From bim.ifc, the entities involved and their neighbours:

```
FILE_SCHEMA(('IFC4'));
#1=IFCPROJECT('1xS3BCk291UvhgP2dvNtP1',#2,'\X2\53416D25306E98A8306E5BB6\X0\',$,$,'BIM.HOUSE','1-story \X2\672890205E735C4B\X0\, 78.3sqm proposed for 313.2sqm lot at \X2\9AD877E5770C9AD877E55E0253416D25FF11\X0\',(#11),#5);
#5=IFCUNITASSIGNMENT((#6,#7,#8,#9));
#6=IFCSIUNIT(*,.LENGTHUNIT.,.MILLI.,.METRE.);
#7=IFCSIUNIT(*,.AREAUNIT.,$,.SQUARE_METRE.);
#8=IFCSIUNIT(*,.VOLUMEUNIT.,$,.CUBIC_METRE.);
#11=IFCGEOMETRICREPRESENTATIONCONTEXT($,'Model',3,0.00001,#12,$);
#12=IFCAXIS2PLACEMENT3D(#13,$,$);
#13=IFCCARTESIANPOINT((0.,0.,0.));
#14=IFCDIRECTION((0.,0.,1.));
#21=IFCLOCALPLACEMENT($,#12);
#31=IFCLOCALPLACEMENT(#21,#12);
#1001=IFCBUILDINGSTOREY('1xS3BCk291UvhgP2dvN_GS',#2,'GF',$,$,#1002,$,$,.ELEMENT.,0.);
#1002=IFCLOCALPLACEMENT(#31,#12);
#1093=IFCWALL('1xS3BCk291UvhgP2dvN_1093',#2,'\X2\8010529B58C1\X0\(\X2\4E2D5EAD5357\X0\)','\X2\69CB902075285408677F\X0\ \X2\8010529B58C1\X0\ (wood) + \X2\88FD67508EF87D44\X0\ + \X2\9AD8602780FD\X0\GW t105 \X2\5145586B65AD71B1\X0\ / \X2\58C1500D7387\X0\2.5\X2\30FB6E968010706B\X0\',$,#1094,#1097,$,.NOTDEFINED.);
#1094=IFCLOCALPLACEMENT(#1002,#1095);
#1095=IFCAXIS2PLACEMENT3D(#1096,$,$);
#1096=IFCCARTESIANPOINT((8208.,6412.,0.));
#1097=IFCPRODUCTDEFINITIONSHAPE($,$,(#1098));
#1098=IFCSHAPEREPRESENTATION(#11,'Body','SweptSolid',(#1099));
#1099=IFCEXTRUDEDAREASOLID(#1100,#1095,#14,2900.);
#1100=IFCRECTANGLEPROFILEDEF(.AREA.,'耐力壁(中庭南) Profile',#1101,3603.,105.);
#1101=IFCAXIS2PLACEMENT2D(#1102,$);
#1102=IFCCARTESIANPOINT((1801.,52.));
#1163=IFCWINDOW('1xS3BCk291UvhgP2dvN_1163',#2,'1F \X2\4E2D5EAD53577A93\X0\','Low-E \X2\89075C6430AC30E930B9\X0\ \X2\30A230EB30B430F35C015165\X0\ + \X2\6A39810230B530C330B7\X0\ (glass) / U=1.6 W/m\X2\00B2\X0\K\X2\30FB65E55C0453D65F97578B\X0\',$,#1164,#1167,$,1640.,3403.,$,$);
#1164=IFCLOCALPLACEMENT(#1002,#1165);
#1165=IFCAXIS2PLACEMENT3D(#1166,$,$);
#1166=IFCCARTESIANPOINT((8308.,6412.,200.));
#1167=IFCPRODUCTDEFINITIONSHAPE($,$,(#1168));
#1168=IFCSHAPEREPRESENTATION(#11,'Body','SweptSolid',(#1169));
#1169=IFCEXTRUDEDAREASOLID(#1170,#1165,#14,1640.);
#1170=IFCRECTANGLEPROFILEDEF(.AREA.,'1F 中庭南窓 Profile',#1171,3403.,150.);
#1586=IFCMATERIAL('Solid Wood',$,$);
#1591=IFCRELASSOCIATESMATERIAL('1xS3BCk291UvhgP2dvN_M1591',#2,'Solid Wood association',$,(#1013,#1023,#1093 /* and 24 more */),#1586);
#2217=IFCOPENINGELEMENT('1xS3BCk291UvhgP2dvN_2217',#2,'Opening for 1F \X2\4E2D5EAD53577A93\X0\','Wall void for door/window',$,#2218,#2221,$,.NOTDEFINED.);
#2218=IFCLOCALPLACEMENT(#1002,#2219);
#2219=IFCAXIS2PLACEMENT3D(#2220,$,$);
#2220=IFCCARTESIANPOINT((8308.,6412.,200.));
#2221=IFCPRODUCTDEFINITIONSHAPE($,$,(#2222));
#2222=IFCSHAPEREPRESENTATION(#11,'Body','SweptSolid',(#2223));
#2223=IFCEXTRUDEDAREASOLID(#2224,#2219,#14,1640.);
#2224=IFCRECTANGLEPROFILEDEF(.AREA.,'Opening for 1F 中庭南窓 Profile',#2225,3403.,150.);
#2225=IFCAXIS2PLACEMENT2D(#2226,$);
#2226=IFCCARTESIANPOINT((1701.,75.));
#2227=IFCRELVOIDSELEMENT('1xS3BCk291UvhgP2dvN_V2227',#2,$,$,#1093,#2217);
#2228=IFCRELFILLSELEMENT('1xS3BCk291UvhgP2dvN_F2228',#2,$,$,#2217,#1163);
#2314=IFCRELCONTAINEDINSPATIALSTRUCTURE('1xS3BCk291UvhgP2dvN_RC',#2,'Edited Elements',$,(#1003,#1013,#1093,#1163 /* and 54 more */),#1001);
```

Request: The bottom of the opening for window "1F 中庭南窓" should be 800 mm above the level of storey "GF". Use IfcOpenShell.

```python
import numpy as np
import ifcopenshell
import ifcopenshell.api.geometry
import ifcopenshell.geom
import ifcopenshell.util.element
import ifcopenshell.util.placement
import ifcopenshell.util.shape
import ifcopenshell.util.unit

model = ifcopenshell.open("bim.ifc")
unit_scale = ifcopenshell.util.unit.calculate_unit_scale(model)

window = model.by_guid("1xS3BCk291UvhgP2dvN_1163")
opening = window.FillsVoids[0].RelatingOpeningElement
storey = ifcopenshell.util.element.get_container(window, ifc_class="IfcBuildingStorey")
level = ifcopenshell.util.placement.get_local_placement(storey.ObjectPlacement)[2, 3]

# The opening's origin need not be at the sill, so measure its lowest point.
shape = ifcopenshell.geom.create_shape(ifcopenshell.geom.settings(), opening)
bottom = ifcopenshell.util.shape.get_shape_bottom_elevation(shape, shape.geometry) / unit_scale
dz = level + 0.8 / unit_scale - bottom

shift = np.array([0.0, 0.0, dz])
# The window is not placed relative to its opening, so move both.
for product in (opening, window):
    matrix = ifcopenshell.util.placement.get_local_placement(product.ObjectPlacement)
    matrix[:3, 3] += shift
    ifcopenshell.api.geometry.edit_object_placement(model, product=product, matrix=matrix, is_si=False)

print(f"moved by {dz * unit_scale:+.3f} m")

model.write("bim_edited.ifc")
```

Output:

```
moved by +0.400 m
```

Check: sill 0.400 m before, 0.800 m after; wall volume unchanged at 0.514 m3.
